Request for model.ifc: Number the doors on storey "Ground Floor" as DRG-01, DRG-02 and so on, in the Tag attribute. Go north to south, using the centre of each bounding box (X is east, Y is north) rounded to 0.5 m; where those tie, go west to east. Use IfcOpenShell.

First a look at what the model holds.

```python
import ifcopenshell
import ifcopenshell.util.element
import ifcopenshell.util.placement

model = ifcopenshell.open("model.ifc")
print(model.schema)
storey = next(s for s in model.by_type("IfcBuildingStorey") if s.Name == "Ground Floor")
doors = [e for e in ifcopenshell.util.element.get_decomposition(storey) if e.is_a("IfcDoor")]
for e in sorted(doors, key=lambda e: e.id()):
    origin = ifcopenshell.util.placement.get_local_placement(e.ObjectPlacement)[:3, 3]
    print(e.id(), e.Tag, e.Name, origin.round(2) + 0.0, sep=" | ")
```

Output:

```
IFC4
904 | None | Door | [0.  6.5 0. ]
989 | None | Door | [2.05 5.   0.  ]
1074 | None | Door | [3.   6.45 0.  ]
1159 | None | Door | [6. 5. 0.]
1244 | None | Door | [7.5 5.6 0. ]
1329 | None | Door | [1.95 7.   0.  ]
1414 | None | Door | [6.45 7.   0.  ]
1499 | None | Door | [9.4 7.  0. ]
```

```python
import ifcopenshell
import ifcopenshell.geom
import ifcopenshell.util.element
import ifcopenshell.util.shape

model = ifcopenshell.open("model.ifc")
settings = ifcopenshell.geom.settings()
settings.set("use-world-coords", True)


def centre(element):
    shape = ifcopenshell.geom.create_shape(settings, element)
    return ifcopenshell.util.shape.get_bbox_centroid(shape.geometry)


storey = next(s for s in model.by_type("IfcBuildingStorey") if s.Name == "Ground Floor")
doors = [e for e in ifcopenshell.util.element.get_decomposition(storey) if e.is_a("IfcDoor")]

# Insertion points can sit at a corner or the storey origin, so sort by the geometry (in metres).
centres = {e: centre(e) for e in doors}
doors.sort(key=lambda e: (-round(centres[e][1] / 0.5), centres[e][0]))

for i, e in enumerate(doors, start=1):
    number = f"DRG-{i:02d}"
    e.Tag = number
    print(e.id(), number)

model.write("model_rev.ifc")
```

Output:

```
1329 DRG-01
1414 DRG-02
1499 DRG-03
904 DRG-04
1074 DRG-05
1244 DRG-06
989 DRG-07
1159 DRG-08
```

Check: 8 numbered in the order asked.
